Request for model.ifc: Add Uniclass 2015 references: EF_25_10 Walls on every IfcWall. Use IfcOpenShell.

First a look at what the model holds.

```python
import ifcopenshell

model = ifcopenshell.open("model.ifc")
print(model.schema)
print("classifications:", [c.Name for c in model.by_type("IfcClassification")])
for ifc_class in ("IfcDoor", "IfcRoof", "IfcStair", "IfcWall", "IfcWindow"):
    print(ifc_class, len(model.by_type(ifc_class)))
```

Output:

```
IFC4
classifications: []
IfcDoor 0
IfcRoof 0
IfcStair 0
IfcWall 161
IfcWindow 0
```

```python
import ifcopenshell
import ifcopenshell.api.classification

model = ifcopenshell.open("model.ifc")

system = ifcopenshell.api.classification.add_classification(model, classification="Uniclass 2015")

codes = {
    "IfcWall": ("EF_25_10", "Walls"),
}
for ifc_class, (code, name) in codes.items():
    products = model.by_type(ifc_class)
    ifcopenshell.api.classification.add_reference(
        model, products=products, classification=system, identification=code, name=name
    )
    print(code, len(products))

model.write("model_updated.ifc")
```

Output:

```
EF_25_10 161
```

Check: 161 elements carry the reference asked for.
